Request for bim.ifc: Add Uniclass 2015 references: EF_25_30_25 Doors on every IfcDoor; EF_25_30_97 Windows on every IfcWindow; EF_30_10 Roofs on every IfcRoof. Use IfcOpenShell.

First a look at what the model holds.

```python
import ifcopenshell

model = ifcopenshell.open("bim.ifc")
print(model.schema)
print("classifications:", [c.Name for c in model.by_type("IfcClassification")])
for ifc_class in ("IfcDoor", "IfcRoof", "IfcStair", "IfcWall", "IfcWindow"):
    print(ifc_class, len(model.by_type(ifc_class)))
```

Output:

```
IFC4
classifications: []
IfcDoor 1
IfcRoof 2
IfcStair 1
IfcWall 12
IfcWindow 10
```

```python
import ifcopenshell
import ifcopenshell.api.classification

model = ifcopenshell.open("bim.ifc")

system = ifcopenshell.api.classification.add_classification(model, classification="Uniclass 2015")

codes = {
    "IfcDoor": ("EF_25_30_25", "Doors"),
    "IfcWindow": ("EF_25_30_97", "Windows"),
    "IfcRoof": ("EF_30_10", "Roofs"),
}
for ifc_class, (code, name) in codes.items():
    products = model.by_type(ifc_class)
    ifcopenshell.api.classification.add_reference(
        model, products=products, classification=system, identification=code, name=name
    )
    print(code, len(products))

model.write("bim_edited.ifc")
```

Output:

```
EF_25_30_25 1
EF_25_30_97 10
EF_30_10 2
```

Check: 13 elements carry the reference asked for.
